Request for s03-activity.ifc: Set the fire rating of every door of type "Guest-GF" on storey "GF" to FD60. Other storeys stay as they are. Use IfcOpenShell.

First a look at what the model holds.

```python
import ifcopenshell
import ifcopenshell.util.element

model = ifcopenshell.open("s03-activity.ifc")
print(model.schema)
storey = next(s for s in model.by_type("IfcBuildingStorey") if s.Name == "GF")
doors = [e for e in ifcopenshell.util.element.get_decomposition(storey) if e.is_a("IfcDoor")]
seen = {}
for e in doors:
    element_type = ifcopenshell.util.element.get_type(e)
    key = (element_type.Name if element_type != e and element_type else None, ifcopenshell.util.element.get_pset(e, "Pset_DoorCommon", "FireRating"))
    seen[key] = seen.get(key, 0) + 1
for (name, value), count in sorted(seen.items(), key=str):
    print(count, "x", name, "|", value)
```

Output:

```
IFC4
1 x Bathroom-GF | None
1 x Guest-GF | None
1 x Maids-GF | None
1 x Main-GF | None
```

```python
import ifcopenshell
import ifcopenshell.api.pset
import ifcopenshell.util.element

model = ifcopenshell.open("s03-activity.ifc")

storey = next(s for s in model.by_type("IfcBuildingStorey") if s.Name == "GF")
doors = [e for e in ifcopenshell.util.element.get_decomposition(storey) if e.is_a("IfcDoor")]

count = 0
for e in doors:
    element_type = ifcopenshell.util.element.get_type(e)
    if element_type in (None, e) or element_type.Name != "Guest-GF":
        continue
    # add_pset returns the element's existing set when there is one.
    pset = ifcopenshell.api.pset.add_pset(model, product=e, name="Pset_DoorCommon")
    ifcopenshell.api.pset.edit_pset(model, pset=pset, properties={"FireRating": "FD60"})
    count += 1

print(count, "doors updated")

model.write("s03-activity-out.ifc")
```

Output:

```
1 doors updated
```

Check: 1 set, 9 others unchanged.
